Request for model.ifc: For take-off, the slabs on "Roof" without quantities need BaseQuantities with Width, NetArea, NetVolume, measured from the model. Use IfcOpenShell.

First a look at what the model holds.

```python
import ifcopenshell
import ifcopenshell.util.element
import ifcopenshell.util.unit

model = ifcopenshell.open("model.ifc")
print(model.schema)
for unit_type in ("LENGTHUNIT", "AREAUNIT", "VOLUMEUNIT"):
    print(unit_type, ifcopenshell.util.unit.calculate_unit_scale(model, unit_type))
storey = next(s for s in model.by_type("IfcBuildingStorey") if s.Name == "Roof")
slabs = [e for e in ifcopenshell.util.element.get_decomposition(storey) if e.is_a("IfcSlab")]
for e in sorted(slabs, key=lambda e: e.id()):
    print(e.id(), e.is_a(), e.Name, list(ifcopenshell.util.element.get_psets(e, qtos_only=True)), sep=" | ")
```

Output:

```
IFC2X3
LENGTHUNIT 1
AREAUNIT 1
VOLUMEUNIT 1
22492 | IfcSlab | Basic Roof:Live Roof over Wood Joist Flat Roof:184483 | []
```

```python
import ifcopenshell
import ifcopenshell.api.pset
import ifcopenshell.geom
import ifcopenshell.util.element
import ifcopenshell.util.shape
import ifcopenshell.util.unit

model = ifcopenshell.open("model.ifc")
unit_scale = ifcopenshell.util.unit.calculate_unit_scale(model)
area_scale = ifcopenshell.util.unit.calculate_unit_scale(model, "AREAUNIT")
volume_scale = ifcopenshell.util.unit.calculate_unit_scale(model, "VOLUMEUNIT")
settings = ifcopenshell.geom.settings()

storey = next(s for s in model.by_type("IfcBuildingStorey") if s.Name == "Roof")
slabs = [e for e in ifcopenshell.util.element.get_decomposition(storey) if e.is_a("IfcSlab")]

for e in sorted(slabs, key=lambda e: e.id()):
    if ifcopenshell.util.element.get_psets(e, qtos_only=True, should_inherit=False):
        continue
    # Geometry comes back in metres, in the element's own axes.
    shape = ifcopenshell.geom.create_shape(settings, e)
    values = {
        "Width": ifcopenshell.util.shape.get_z(shape.geometry) / unit_scale,
        "NetArea": ifcopenshell.util.shape.get_footprint_area(shape.geometry) / area_scale,
        "NetVolume": ifcopenshell.util.shape.get_volume(shape.geometry) / volume_scale,
    }
    qto = ifcopenshell.api.pset.add_qto(model, product=e, name="BaseQuantities")
    ifcopenshell.api.pset.edit_qto(model, qto=qto, properties=values)
    print(e.id(), {k: round(v, 3) for k, v in values.items()})

model.write("model_rev.ifc")
```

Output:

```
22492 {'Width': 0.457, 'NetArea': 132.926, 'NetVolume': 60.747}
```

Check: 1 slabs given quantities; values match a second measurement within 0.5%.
